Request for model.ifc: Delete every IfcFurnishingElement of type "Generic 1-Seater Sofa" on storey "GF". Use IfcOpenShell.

First a look at what the model holds.

```python
import ifcopenshell
import ifcopenshell.util.element

model = ifcopenshell.open("model.ifc")
print(model.schema)
storey = next(s for s in model.by_type("IfcBuildingStorey") if s.Name == "GF")
furniture = [e for e in ifcopenshell.util.element.get_decomposition(storey) if e.is_a("IfcFurnishingElement")]
seen = {}
for e in furniture:
    element_type = ifcopenshell.util.element.get_type(e)
    name = element_type.Name if element_type not in (None, e) else None
    seen[name] = seen.get(name, 0) + 1
for name, count in sorted(seen.items(), key=str):
    print(count, "x", name)
```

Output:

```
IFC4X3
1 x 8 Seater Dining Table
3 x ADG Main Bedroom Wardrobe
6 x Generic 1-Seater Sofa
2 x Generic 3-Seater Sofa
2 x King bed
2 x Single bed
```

```python
import ifcopenshell
import ifcopenshell.api.root
import ifcopenshell.util.element

model = ifcopenshell.open("model.ifc")

storey = next(s for s in model.by_type("IfcBuildingStorey") if s.Name == "GF")
furniture = [e for e in ifcopenshell.util.element.get_decomposition(storey) if e.is_a("IfcFurnishingElement")]
targets = [e for e in furniture if (t := ifcopenshell.util.element.get_type(e)) not in (None, e) and t.Name == "Generic 1-Seater Sofa"]

for e in targets:
    ifcopenshell.api.root.remove_product(model, product=e)
print(len(targets), "removed")

model.write("model_v2.ifc")
```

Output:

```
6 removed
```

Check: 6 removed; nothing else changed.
